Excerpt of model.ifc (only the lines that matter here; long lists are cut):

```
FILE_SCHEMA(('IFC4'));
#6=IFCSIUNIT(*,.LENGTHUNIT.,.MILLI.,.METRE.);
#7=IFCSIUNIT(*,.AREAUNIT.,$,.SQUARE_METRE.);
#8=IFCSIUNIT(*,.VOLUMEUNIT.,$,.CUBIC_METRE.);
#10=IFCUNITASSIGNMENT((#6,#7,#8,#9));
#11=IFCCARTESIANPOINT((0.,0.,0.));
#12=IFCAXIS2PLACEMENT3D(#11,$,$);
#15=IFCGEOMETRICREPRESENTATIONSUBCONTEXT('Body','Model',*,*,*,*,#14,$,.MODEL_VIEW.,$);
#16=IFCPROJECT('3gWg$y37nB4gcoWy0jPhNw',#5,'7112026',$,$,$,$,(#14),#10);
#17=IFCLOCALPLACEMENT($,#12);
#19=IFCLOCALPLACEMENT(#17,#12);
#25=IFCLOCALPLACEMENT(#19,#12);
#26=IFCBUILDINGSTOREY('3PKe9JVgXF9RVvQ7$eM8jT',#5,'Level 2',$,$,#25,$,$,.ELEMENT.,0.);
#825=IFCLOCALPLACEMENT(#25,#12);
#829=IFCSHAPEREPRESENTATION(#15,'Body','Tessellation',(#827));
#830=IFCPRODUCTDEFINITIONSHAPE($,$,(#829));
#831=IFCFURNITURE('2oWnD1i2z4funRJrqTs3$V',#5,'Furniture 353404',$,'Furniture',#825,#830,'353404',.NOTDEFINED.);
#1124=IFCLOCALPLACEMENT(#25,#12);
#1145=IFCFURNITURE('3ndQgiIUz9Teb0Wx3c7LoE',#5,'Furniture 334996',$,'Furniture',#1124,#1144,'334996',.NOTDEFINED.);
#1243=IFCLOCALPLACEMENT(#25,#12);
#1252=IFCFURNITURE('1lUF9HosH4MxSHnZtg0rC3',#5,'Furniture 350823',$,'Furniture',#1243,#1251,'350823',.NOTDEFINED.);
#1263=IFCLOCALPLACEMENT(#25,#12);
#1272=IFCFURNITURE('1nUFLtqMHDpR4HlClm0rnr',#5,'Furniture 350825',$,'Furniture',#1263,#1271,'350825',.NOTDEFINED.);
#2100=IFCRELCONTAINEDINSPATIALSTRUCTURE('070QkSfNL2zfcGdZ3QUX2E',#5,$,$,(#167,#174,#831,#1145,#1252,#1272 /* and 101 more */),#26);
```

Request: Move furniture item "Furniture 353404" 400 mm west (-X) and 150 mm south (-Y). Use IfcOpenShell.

```python
import ifcopenshell
import ifcopenshell.api.geometry
import ifcopenshell.util.placement
import ifcopenshell.util.unit

model = ifcopenshell.open("model.ifc")
unit_scale = ifcopenshell.util.unit.calculate_unit_scale(model)

item = model.by_guid("2oWnD1i2z4funRJrqTs3$V")
matrix = ifcopenshell.util.placement.get_local_placement(item.ObjectPlacement)
matrix[0, 3] -= 0.4 / unit_scale
matrix[1, 3] -= 0.15 / unit_scale
ifcopenshell.api.geometry.edit_object_placement(model, product=item, matrix=matrix, is_si=False)

print(ifcopenshell.util.placement.get_local_placement(item.ObjectPlacement).round(3) + 0.0)

model.write("model_v2.ifc")
```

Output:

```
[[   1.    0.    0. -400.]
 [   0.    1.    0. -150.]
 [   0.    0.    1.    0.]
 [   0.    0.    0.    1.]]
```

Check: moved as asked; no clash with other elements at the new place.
